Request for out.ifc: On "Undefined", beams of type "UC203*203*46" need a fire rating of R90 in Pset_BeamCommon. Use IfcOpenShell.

First a look at what the model holds.

```python
import ifcopenshell
import ifcopenshell.util.element

model = ifcopenshell.open("out.ifc")
print(model.schema)
storey = next(s for s in model.by_type("IfcBuildingStorey") if s.Name == "Undefined")
beams = [e for e in ifcopenshell.util.element.get_decomposition(storey) if e.is_a("IfcBeam")]
seen = {}
for e in beams:
    element_type = ifcopenshell.util.element.get_type(e)
    key = (element_type.Name if element_type != e and element_type else None, ifcopenshell.util.element.get_pset(e, "Pset_BeamCommon", "FireRating"))
    seen[key] = seen.get(key, 0) + 1
for (name, value), count in sorted(seen.items(), key=str):
    print(count, "x", name, "|", value)
```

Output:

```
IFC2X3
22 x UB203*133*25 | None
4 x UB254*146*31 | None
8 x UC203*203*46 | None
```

```python
import ifcopenshell
import ifcopenshell.api.pset
import ifcopenshell.util.element

model = ifcopenshell.open("out.ifc")

storey = next(s for s in model.by_type("IfcBuildingStorey") if s.Name == "Undefined")
beams = [e for e in ifcopenshell.util.element.get_decomposition(storey) if e.is_a("IfcBeam")]

count = 0
for e in beams:
    element_type = ifcopenshell.util.element.get_type(e)
    if element_type in (None, e) or element_type.Name != "UC203*203*46":
        continue
    found = ifcopenshell.util.element.get_pset(e, "Pset_BeamCommon", should_inherit=False)
    if found:
        pset = model.by_id(found["id"])
        if len(ifcopenshell.util.element.get_elements_by_pset(pset)) > 1:
            pset = ifcopenshell.api.pset.unshare_pset(model, products=[e], pset=pset)[0]
    else:
        pset = ifcopenshell.api.pset.add_pset(model, product=e, name="Pset_BeamCommon")
    ifcopenshell.api.pset.edit_pset(model, pset=pset, properties={"FireRating": "R90"})
    count += 1

print(count, "beams updated")

model.write("out_rev.ifc")
```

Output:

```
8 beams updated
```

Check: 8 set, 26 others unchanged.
